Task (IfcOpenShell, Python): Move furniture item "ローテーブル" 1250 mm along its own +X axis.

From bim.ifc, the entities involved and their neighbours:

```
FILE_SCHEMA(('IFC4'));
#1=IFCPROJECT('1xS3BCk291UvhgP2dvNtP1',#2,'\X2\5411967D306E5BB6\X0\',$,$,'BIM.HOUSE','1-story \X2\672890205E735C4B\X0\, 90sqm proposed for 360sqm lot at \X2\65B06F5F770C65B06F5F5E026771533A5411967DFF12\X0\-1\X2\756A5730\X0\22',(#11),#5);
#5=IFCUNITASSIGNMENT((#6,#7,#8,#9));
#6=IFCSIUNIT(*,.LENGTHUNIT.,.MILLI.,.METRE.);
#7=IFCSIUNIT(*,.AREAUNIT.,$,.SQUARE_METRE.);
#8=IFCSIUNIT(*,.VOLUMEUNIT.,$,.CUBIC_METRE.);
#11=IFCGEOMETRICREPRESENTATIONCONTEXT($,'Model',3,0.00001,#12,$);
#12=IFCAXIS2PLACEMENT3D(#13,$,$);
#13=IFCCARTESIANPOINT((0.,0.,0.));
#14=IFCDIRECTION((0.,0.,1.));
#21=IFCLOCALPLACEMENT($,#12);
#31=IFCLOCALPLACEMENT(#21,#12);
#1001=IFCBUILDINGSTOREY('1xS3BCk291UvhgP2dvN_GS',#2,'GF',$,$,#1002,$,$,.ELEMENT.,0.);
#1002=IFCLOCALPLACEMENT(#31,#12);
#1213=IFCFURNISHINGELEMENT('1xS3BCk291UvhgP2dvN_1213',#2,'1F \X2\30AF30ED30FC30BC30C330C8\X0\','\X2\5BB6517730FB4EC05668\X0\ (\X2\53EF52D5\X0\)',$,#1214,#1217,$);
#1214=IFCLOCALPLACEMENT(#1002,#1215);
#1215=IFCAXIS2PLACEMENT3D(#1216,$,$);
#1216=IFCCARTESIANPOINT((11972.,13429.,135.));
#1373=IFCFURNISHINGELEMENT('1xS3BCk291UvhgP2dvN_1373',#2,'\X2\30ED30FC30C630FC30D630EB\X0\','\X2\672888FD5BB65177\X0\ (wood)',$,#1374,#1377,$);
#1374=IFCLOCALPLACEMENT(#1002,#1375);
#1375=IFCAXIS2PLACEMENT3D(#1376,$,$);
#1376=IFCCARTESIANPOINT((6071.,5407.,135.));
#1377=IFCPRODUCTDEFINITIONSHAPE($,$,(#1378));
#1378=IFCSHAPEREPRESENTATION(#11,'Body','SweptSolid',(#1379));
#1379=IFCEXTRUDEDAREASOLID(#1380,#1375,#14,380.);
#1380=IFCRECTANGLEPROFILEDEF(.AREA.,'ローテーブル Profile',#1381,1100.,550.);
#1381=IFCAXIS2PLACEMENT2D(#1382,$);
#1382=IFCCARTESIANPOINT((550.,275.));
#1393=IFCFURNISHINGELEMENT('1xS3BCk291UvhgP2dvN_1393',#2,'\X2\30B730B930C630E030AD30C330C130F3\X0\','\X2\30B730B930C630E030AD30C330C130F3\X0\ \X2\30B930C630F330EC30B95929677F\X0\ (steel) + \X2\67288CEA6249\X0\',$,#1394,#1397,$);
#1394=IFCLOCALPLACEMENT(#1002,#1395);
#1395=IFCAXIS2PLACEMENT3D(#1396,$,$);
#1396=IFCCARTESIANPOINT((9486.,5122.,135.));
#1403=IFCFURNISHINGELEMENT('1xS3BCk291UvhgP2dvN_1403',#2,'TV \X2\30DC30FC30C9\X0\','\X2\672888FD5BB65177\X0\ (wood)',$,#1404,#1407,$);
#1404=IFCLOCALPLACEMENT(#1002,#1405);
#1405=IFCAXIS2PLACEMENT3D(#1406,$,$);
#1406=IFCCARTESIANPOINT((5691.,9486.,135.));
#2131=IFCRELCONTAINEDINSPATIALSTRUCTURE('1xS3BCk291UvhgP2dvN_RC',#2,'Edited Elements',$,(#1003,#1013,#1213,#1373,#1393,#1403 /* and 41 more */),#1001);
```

```python
import ifcopenshell
import ifcopenshell.api.geometry
import ifcopenshell.util.placement
import ifcopenshell.util.unit

model = ifcopenshell.open("bim.ifc")
unit_scale = ifcopenshell.util.unit.calculate_unit_scale(model)

item = model.by_guid("1xS3BCk291UvhgP2dvN_1373")
matrix = ifcopenshell.util.placement.get_local_placement(item.ObjectPlacement)
matrix[:3, 3] += matrix[:3, 0] * 1.25 / unit_scale
ifcopenshell.api.geometry.edit_object_placement(model, product=item, matrix=matrix, is_si=False)

print(ifcopenshell.util.placement.get_local_placement(item.ObjectPlacement).round(3) + 0.0)

model.write("bim_updated.ifc")
```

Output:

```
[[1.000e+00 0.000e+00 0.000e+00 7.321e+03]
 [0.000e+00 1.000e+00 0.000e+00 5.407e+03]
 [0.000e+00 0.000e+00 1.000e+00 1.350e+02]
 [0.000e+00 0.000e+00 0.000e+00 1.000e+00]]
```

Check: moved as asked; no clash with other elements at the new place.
